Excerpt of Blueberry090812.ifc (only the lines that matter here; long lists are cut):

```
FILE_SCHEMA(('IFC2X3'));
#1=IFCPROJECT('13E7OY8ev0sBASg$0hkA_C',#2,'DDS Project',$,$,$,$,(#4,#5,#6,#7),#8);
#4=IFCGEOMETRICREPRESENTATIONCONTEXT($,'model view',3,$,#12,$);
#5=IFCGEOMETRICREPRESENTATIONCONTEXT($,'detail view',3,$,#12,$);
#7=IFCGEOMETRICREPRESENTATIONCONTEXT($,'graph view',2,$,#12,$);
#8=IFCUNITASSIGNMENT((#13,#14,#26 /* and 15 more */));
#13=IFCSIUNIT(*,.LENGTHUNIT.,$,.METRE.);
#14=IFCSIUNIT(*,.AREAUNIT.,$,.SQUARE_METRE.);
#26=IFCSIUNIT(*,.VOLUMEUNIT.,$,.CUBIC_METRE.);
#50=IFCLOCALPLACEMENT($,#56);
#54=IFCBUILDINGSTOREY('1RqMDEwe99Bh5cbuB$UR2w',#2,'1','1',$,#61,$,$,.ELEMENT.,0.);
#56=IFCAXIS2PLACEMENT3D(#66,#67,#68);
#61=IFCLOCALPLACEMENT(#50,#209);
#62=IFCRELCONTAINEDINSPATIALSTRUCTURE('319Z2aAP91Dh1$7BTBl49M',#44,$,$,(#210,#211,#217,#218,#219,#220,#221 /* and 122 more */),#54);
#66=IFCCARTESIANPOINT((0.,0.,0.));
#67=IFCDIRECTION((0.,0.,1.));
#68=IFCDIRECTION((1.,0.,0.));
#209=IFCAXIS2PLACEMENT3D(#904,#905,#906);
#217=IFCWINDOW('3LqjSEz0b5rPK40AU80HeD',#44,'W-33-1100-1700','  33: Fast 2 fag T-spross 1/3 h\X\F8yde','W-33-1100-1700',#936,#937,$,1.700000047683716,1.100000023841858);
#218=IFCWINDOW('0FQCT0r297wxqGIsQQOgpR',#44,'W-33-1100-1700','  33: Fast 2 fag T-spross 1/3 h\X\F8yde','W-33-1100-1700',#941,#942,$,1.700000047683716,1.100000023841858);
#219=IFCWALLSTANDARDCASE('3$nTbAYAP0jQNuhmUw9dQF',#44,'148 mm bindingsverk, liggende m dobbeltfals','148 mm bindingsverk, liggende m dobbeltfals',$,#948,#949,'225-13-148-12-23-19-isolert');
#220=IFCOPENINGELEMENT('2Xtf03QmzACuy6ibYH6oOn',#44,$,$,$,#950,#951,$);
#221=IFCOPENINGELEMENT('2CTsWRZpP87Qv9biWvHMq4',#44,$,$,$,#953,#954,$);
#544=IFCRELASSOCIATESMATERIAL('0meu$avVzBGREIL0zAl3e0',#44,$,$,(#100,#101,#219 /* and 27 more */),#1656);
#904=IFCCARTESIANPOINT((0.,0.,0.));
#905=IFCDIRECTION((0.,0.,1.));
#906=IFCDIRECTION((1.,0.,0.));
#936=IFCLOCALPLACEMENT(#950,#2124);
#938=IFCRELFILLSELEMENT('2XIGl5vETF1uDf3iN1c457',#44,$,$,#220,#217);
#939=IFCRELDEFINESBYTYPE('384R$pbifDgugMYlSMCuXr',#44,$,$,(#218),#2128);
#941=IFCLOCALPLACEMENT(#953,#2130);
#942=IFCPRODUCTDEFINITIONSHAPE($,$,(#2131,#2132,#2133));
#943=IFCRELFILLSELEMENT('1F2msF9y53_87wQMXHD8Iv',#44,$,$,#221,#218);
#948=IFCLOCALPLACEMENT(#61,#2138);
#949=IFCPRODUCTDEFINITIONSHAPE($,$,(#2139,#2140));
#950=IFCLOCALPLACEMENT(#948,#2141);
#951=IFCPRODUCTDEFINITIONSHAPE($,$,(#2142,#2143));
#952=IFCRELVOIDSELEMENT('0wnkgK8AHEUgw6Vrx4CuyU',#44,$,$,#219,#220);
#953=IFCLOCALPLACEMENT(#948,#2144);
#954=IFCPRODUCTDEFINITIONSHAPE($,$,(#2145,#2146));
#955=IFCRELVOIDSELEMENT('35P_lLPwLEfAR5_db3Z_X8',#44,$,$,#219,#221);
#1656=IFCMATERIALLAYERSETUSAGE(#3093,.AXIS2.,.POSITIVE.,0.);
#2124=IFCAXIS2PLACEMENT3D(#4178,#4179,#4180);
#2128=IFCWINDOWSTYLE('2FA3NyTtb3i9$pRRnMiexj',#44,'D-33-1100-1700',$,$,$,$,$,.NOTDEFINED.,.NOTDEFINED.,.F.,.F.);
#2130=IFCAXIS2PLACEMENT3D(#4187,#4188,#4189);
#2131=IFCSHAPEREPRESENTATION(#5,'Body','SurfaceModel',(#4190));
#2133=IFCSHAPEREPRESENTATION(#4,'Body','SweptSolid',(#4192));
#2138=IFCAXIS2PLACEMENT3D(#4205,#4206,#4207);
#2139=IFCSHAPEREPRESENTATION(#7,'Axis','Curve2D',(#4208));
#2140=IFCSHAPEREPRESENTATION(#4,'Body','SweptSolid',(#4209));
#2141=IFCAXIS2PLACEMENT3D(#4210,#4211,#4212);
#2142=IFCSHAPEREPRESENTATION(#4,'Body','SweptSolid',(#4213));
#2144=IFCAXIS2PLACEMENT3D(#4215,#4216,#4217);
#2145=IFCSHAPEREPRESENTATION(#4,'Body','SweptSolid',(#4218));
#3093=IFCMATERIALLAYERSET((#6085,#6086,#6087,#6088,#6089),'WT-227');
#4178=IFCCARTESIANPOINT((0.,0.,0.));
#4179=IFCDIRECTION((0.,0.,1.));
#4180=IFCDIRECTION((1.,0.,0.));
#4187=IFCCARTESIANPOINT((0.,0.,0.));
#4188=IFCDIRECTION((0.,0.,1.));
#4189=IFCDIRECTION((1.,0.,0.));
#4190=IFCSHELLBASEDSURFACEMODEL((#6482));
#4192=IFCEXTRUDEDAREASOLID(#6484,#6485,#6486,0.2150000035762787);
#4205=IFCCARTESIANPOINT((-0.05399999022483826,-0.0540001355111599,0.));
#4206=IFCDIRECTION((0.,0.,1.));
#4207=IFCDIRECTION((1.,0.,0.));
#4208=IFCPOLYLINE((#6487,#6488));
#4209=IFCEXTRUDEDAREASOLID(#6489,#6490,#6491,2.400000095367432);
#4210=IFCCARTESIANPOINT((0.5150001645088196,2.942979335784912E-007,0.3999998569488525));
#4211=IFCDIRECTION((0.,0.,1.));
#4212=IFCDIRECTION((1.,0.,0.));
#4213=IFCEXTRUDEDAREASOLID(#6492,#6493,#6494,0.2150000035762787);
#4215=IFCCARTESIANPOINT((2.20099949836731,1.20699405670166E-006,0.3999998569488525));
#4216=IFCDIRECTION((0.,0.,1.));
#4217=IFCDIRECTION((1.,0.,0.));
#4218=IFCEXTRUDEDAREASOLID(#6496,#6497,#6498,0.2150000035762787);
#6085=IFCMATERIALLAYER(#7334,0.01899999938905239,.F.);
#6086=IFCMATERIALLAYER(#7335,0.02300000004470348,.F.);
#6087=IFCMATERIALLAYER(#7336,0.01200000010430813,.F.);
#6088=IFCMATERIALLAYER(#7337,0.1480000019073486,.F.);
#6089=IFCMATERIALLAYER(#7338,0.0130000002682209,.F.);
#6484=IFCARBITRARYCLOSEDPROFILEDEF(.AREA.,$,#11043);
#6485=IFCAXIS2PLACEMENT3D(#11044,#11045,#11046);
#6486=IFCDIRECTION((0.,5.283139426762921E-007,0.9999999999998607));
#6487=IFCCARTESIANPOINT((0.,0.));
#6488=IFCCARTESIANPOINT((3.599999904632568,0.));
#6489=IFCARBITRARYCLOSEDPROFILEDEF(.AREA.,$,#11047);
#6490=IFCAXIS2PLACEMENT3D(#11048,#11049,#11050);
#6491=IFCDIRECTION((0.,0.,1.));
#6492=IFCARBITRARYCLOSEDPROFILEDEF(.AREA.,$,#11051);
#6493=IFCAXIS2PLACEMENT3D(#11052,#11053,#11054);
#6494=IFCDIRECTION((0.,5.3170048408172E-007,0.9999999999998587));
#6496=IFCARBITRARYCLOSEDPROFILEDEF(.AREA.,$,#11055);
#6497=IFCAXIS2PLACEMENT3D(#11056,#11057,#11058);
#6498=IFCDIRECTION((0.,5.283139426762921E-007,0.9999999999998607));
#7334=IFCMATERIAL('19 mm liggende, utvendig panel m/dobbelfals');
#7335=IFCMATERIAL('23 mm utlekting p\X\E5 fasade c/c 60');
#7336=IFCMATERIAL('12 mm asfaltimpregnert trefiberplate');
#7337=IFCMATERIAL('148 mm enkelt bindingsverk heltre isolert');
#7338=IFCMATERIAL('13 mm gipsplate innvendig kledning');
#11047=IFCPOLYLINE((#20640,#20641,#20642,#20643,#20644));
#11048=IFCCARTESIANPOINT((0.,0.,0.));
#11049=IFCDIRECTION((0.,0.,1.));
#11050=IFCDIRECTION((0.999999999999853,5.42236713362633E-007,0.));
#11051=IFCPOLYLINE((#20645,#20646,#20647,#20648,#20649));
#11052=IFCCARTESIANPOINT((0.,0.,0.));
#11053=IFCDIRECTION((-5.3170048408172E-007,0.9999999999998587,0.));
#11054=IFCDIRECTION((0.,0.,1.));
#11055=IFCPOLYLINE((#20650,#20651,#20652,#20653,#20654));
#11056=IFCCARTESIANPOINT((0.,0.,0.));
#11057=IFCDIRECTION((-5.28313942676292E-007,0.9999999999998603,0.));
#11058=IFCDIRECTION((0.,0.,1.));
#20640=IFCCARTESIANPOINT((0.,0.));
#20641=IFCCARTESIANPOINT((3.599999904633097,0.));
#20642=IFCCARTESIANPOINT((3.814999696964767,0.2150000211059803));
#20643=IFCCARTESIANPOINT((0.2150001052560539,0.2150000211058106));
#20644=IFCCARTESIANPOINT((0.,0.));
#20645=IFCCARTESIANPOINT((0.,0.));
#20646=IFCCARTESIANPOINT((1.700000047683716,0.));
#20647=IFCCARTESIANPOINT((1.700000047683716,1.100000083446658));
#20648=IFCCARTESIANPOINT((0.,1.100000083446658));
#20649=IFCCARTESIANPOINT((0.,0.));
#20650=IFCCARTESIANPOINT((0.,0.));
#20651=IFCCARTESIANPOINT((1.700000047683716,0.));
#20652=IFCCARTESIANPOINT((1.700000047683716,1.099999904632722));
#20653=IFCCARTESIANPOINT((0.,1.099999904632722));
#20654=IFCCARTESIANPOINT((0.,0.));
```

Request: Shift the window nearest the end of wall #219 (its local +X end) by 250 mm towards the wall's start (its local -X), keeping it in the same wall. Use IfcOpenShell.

```python
import ifcopenshell
import ifcopenshell.api.geometry
import ifcopenshell.util.placement

model = ifcopenshell.open("Blueberry090812.ifc")

window = model.by_guid("0FQCT0r297wxqGIsQQOgpR")
opening = window.FillsVoids[0].RelatingOpeningElement
wall = opening.VoidsElements[0].RelatingBuildingElement

wall_matrix = ifcopenshell.util.placement.get_local_placement(wall.ObjectPlacement)
shift = wall_matrix[:3, 0] * -0.25
before = ifcopenshell.util.placement.get_local_placement(window.ObjectPlacement)[:3, 3].copy()

# The window is placed relative to its opening, so it follows when the opening moves.
matrix = ifcopenshell.util.placement.get_local_placement(opening.ObjectPlacement)
matrix[:3, 3] += shift
ifcopenshell.api.geometry.edit_object_placement(
    model, product=opening, matrix=matrix, is_si=False, should_transform_children=True
)

after = ifcopenshell.util.placement.get_local_placement(window.ObjectPlacement)[:3, 3]
print("window moved by", (after - before).round(3) + 0.0)

model.write("Blueberry090812_edited.ifc")
```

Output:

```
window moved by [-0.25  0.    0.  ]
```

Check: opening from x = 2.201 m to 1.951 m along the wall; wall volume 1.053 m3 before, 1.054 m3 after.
